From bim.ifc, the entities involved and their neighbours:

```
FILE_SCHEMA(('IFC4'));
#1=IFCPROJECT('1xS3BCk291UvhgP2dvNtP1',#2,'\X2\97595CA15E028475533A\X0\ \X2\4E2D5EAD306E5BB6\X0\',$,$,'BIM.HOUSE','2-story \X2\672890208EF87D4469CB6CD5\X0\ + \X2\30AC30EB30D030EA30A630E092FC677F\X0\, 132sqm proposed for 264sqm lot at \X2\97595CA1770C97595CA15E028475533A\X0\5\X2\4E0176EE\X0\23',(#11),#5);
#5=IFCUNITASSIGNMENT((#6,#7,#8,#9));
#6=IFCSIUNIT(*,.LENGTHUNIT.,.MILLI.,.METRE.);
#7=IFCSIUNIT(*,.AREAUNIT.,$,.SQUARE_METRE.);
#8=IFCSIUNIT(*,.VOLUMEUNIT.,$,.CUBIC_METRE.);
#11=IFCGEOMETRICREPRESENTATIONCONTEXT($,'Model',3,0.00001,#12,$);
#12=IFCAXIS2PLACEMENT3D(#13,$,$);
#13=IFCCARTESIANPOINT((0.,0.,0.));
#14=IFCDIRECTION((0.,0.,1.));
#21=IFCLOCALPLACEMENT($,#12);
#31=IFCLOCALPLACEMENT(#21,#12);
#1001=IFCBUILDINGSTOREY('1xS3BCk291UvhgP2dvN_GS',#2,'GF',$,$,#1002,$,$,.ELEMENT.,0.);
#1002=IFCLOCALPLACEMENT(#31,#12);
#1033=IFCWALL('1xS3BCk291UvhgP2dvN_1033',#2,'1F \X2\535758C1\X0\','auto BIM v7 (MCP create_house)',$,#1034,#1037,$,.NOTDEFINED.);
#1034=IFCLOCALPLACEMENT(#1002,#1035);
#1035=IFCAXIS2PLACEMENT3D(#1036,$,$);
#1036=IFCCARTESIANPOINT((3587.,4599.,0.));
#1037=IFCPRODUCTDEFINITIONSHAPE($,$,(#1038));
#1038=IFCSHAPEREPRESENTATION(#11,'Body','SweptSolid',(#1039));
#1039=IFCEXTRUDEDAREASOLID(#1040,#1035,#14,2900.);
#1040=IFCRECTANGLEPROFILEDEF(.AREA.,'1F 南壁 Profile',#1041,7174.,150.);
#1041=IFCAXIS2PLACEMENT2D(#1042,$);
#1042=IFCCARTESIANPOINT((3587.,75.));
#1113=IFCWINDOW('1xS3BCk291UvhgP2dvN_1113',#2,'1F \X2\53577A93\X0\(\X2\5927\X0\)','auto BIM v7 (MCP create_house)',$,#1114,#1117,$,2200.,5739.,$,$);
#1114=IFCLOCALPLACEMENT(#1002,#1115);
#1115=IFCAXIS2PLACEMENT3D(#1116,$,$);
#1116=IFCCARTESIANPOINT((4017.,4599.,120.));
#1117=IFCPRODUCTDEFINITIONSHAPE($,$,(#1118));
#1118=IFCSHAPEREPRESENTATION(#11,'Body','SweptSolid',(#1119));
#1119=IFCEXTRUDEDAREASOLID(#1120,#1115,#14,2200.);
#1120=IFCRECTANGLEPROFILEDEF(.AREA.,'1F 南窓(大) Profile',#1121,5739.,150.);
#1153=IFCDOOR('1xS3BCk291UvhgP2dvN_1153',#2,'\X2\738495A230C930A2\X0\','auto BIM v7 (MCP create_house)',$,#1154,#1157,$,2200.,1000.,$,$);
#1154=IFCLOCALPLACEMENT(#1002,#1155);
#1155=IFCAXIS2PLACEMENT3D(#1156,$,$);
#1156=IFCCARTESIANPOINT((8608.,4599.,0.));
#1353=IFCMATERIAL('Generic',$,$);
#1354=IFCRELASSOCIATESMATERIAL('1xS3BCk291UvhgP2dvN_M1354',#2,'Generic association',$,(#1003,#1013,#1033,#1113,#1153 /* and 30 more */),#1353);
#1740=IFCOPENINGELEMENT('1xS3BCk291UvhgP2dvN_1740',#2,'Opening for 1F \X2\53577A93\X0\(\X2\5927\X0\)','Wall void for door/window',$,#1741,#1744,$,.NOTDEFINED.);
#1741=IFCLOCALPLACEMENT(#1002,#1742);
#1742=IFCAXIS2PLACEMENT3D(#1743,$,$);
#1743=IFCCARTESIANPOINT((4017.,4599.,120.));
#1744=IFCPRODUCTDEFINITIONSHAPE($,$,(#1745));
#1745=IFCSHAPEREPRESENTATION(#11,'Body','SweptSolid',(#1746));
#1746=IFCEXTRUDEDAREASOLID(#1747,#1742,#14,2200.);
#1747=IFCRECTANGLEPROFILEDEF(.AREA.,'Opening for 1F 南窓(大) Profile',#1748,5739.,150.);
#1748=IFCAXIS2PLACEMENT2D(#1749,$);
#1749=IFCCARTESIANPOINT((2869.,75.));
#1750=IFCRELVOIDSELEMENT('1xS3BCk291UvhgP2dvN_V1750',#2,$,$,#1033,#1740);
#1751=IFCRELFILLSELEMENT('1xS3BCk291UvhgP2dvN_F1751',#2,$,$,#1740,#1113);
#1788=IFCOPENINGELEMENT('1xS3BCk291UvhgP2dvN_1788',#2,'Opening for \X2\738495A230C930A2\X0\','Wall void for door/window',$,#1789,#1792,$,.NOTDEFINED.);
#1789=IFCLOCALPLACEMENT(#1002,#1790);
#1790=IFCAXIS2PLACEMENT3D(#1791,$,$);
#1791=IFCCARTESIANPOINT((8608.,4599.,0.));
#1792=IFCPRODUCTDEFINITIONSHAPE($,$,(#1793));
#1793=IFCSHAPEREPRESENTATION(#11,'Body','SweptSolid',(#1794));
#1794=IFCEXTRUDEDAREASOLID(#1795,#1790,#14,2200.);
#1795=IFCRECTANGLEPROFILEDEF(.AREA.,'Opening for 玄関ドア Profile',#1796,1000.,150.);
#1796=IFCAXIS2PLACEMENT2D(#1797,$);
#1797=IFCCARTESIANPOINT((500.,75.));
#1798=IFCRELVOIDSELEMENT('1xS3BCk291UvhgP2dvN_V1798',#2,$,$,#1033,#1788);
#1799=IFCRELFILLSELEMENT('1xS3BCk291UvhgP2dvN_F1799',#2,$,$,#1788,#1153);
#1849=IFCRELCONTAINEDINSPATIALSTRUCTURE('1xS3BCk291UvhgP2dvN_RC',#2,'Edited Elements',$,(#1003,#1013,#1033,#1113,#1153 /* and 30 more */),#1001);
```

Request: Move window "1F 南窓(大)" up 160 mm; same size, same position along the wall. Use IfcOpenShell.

```python
import numpy as np
import ifcopenshell
import ifcopenshell.api.geometry
import ifcopenshell.util.placement
import ifcopenshell.util.unit

model = ifcopenshell.open("bim.ifc")
unit_scale = ifcopenshell.util.unit.calculate_unit_scale(model)

window = model.by_id(1113)
opening = window.FillsVoids[0].RelatingOpeningElement
dz = 0.16 / unit_scale

shift = np.array([0.0, 0.0, dz])
# The window is not placed relative to its opening, so move both.
for product in (opening, window):
    matrix = ifcopenshell.util.placement.get_local_placement(product.ObjectPlacement)
    matrix[:3, 3] += shift
    ifcopenshell.api.geometry.edit_object_placement(model, product=product, matrix=matrix, is_si=False)

print(f"moved by {dz * unit_scale:+.3f} m")

model.write("bim-out.ifc")
```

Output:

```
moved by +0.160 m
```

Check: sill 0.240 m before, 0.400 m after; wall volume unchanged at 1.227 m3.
